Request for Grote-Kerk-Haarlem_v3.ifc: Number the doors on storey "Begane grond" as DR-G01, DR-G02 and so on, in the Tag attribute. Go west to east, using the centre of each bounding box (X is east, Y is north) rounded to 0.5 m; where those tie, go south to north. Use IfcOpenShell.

First a look at what the model holds.

```python
import ifcopenshell
import ifcopenshell.util.element
import ifcopenshell.util.placement

model = ifcopenshell.open("Grote-Kerk-Haarlem_v3.ifc")
print(model.schema)
storey = next(s for s in model.by_type("IfcBuildingStorey") if s.Name == "Begane grond")
doors = [e for e in ifcopenshell.util.element.get_decomposition(storey) if e.is_a("IfcDoor")]
for e in sorted(doors, key=lambda e: e.id()):
    origin = ifcopenshell.util.placement.get_local_placement(e.ObjectPlacement)[:3, 3]
    print(e.id(), e.Tag, e.Name, origin.round(2) + 0.0, sep=" | ")
```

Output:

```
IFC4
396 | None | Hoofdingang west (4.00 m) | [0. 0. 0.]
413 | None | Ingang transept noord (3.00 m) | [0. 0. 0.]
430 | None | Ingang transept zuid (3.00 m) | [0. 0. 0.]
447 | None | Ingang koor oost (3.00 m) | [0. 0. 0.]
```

```python
import ifcopenshell
import ifcopenshell.geom
import ifcopenshell.util.element
import ifcopenshell.util.shape

model = ifcopenshell.open("Grote-Kerk-Haarlem_v3.ifc")
settings = ifcopenshell.geom.settings()
settings.set("use-world-coords", True)


def centre(element):
    shape = ifcopenshell.geom.create_shape(settings, element)
    return ifcopenshell.util.shape.get_bbox_centroid(shape.geometry)


storey = next(s for s in model.by_type("IfcBuildingStorey") if s.Name == "Begane grond")
doors = [e for e in ifcopenshell.util.element.get_decomposition(storey) if e.is_a("IfcDoor")]

# Insertion points can sit at a corner or the storey origin, so sort by the geometry (in metres).
centres = {e: centre(e) for e in doors}
doors.sort(key=lambda e: (round(centres[e][0] / 0.5), centres[e][1]))

for i, e in enumerate(doors, start=1):
    number = f"DR-G{i:02d}"
    e.Tag = number
    print(e.id(), number)

model.write("Grote-Kerk-Haarlem_v3_v2.ifc")
```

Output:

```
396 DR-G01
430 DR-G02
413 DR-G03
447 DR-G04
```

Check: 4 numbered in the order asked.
